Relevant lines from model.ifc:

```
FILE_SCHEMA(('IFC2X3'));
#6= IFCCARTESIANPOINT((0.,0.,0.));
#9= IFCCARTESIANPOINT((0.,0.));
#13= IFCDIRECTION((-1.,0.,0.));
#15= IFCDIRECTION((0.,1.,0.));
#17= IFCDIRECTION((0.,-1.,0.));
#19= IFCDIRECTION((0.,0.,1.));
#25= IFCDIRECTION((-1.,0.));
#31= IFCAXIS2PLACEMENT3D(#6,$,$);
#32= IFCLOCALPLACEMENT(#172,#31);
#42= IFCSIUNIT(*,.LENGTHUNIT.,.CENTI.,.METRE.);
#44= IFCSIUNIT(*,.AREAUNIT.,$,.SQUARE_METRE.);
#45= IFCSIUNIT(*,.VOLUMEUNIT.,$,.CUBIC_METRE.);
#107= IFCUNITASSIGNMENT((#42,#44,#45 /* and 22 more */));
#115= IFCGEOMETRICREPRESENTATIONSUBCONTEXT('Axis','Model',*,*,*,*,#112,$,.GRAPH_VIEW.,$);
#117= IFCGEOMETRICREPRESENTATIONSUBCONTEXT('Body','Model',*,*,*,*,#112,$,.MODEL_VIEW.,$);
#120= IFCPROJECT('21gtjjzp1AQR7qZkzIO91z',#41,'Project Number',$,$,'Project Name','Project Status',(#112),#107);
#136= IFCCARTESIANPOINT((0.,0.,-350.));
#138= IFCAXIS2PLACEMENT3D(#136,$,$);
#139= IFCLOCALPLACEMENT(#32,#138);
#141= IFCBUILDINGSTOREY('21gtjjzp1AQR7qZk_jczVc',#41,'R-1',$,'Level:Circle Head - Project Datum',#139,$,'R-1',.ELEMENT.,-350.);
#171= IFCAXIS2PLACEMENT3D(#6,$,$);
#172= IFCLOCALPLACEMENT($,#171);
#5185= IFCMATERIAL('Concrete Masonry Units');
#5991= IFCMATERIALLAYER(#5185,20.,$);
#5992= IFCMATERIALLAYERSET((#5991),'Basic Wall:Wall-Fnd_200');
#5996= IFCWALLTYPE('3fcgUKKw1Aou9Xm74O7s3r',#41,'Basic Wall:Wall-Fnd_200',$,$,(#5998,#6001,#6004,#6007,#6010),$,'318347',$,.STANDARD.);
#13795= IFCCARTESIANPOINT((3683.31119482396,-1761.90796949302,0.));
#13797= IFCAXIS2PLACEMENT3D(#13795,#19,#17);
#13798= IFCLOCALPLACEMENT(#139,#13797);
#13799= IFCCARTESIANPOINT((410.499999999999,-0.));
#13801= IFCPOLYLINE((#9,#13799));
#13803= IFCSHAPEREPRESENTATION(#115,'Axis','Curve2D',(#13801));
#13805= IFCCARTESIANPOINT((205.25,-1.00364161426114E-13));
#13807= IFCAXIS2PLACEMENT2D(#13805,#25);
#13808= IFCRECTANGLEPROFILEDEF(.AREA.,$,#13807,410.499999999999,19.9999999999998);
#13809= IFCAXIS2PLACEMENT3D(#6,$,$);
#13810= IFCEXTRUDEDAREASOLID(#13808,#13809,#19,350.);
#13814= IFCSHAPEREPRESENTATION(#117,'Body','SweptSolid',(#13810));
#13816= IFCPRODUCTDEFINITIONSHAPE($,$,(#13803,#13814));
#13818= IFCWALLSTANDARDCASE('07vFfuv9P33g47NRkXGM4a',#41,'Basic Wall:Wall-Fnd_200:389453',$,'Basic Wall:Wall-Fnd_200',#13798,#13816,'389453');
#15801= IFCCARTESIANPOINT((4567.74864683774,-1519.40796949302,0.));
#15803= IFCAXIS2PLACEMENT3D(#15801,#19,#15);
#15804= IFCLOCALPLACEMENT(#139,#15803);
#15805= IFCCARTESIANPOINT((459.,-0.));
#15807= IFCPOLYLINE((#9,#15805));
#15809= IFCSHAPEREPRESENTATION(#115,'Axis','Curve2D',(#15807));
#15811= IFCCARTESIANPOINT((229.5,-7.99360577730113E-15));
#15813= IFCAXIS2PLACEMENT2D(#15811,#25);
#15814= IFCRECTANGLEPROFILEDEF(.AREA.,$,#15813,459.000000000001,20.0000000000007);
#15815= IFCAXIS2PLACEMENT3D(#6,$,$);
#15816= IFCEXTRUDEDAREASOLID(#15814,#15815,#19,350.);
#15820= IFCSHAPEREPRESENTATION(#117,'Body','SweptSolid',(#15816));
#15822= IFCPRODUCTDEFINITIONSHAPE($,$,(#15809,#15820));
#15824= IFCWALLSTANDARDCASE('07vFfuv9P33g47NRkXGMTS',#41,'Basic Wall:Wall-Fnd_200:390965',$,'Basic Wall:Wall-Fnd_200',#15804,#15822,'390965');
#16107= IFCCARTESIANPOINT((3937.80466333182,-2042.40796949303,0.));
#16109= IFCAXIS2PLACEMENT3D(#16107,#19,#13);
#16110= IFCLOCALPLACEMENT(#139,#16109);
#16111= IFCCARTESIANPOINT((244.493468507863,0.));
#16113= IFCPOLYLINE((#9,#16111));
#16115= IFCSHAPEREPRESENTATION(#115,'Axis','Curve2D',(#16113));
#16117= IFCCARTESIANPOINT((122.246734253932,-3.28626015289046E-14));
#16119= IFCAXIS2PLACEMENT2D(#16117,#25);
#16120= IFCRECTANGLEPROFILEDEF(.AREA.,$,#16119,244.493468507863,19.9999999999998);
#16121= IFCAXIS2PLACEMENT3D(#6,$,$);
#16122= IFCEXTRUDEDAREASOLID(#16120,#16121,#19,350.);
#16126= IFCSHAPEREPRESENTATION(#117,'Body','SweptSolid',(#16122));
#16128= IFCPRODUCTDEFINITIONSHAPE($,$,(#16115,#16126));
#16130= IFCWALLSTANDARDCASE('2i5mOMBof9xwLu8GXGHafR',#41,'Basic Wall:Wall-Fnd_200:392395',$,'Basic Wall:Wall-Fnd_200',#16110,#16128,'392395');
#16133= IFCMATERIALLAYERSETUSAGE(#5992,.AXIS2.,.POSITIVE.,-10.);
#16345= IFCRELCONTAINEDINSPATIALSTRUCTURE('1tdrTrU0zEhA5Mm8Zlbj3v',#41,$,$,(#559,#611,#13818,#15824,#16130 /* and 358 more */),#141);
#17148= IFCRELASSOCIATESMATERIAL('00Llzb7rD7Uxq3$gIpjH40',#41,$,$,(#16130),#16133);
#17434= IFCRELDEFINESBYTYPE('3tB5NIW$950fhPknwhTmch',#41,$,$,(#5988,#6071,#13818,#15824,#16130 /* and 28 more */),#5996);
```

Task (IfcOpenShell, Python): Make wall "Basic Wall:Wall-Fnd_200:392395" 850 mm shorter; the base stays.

```python
import ifcopenshell
import ifcopenshell.geom
import ifcopenshell.util.representation
import ifcopenshell.util.shape
import ifcopenshell.util.unit

model = ifcopenshell.open("model.ifc")
unit_scale = ifcopenshell.util.unit.calculate_unit_scale(model)
settings = ifcopenshell.geom.settings()


def volume(element):
    """Net volume in cubic metres, openings subtracted."""
    shape = ifcopenshell.geom.create_shape(settings, element)
    return ifcopenshell.util.shape.get_volume(shape.geometry)


wall = model.by_guid("2i5mOMBof9xwLu8GXGHafR")
before = volume(wall)

body = ifcopenshell.util.representation.get_representation(wall, "Model", "Body")
solid = body.Items[0]
old_height = solid.Depth
solid.Depth -= 0.85 / unit_scale
after = volume(wall)

print(f"height {old_height:g} -> {solid.Depth:g}, volume {before:.3f} -> {after:.3f} m3")

model.write("model_updated.ifc")
```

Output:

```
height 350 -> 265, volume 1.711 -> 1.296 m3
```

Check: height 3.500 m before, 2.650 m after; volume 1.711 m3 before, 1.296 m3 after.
